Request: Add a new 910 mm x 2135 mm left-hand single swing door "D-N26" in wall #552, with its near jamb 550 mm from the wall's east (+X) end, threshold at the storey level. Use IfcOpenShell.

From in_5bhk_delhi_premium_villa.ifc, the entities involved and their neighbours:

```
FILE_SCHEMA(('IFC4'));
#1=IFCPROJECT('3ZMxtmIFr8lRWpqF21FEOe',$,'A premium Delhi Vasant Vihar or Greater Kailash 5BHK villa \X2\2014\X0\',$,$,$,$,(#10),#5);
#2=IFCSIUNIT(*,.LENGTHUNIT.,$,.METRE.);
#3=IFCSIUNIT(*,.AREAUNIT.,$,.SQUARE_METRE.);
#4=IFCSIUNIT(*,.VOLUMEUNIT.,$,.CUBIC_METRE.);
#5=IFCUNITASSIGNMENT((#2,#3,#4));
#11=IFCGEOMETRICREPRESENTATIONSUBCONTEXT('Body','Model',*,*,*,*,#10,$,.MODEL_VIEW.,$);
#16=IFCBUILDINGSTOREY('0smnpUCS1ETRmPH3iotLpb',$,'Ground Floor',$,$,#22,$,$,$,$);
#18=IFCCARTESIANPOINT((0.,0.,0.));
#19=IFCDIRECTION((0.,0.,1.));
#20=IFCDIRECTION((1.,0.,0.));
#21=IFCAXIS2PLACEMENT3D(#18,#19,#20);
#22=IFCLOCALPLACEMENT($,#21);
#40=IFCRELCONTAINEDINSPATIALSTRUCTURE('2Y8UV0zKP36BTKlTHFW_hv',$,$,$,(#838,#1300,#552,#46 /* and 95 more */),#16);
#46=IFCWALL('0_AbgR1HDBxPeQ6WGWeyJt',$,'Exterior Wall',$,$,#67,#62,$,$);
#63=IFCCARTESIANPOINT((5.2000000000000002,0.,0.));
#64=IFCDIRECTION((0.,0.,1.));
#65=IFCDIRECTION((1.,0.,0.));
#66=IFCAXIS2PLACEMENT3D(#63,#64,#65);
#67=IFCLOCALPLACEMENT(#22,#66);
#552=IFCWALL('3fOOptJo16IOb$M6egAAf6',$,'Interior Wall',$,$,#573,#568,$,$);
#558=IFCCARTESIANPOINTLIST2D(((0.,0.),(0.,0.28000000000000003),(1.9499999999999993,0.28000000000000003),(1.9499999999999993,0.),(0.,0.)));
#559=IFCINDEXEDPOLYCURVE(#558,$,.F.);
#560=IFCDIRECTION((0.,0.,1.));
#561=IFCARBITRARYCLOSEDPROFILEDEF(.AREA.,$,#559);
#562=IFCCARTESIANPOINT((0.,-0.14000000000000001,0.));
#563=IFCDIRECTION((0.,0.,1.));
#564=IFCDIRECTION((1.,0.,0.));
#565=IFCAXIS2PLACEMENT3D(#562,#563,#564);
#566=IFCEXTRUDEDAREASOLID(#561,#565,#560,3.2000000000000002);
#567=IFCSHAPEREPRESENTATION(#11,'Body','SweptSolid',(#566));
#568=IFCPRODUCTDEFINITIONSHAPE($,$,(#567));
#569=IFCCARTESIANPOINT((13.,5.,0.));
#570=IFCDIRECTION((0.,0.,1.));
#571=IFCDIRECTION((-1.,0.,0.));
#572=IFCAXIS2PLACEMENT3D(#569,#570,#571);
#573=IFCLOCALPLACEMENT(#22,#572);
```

```python
import numpy as np
import ifcopenshell
import ifcopenshell.api.feature
import ifcopenshell.api.geometry
import ifcopenshell.api.root
import ifcopenshell.api.spatial
import ifcopenshell.geom
import ifcopenshell.util.element
import ifcopenshell.util.placement
import ifcopenshell.util.representation
import ifcopenshell.util.shape
import ifcopenshell.util.unit

model = ifcopenshell.open("in_5bhk_delhi_premium_villa.ifc")
unit_scale = ifcopenshell.util.unit.calculate_unit_scale(model)
settings = ifcopenshell.geom.settings()


def volume(element):
    """Net volume in cubic metres, openings subtracted."""
    shape = ifcopenshell.geom.create_shape(settings, element)
    return ifcopenshell.util.shape.get_volume(shape.geometry)


wall = model.by_id(552)
storey = ifcopenshell.util.element.get_container(wall, ifc_class="IfcBuildingStorey")
context = ifcopenshell.util.representation.get_context(model, "Model", "Body", "MODEL_VIEW")
before = volume(wall)

width, height, from_end, sill = 0.91, 2.135, 0.55, 0.0  # metres

# The wall runs along its own X axis, and the end named is its -X end.
wall_shape = ifcopenshell.geom.create_shape(settings, wall)
x, y, z = ifcopenshell.util.shape.get_vertices(wall_shape.geometry).T
start = x.min() + from_end
face, thickness = float(y.min()), float(y.max() - y.min())
wall_matrix = ifcopenshell.util.placement.get_local_placement(wall.ObjectPlacement)
level = ifcopenshell.util.placement.get_local_placement(storey.ObjectPlacement)[2, 3]


def in_wall(x, y):
    """Placement at x, y metres in the wall's axes, at sill height."""
    matrix = wall_matrix.copy()
    matrix[:, 3] = wall_matrix @ np.array([x / unit_scale, y / unit_scale, 0.0, 1.0])
    matrix[2, 3] = level + sill / unit_scale
    return matrix


# Opening: a box that overshoots both wall faces by 50 mm.
opening = ifcopenshell.api.root.create_entity(model, ifc_class="IfcOpeningElement", predefined_type="OPENING")
box = ifcopenshell.api.geometry.add_wall_representation(
    model, context=context, length=width, height=height, thickness=thickness + 0.1
)
ifcopenshell.api.geometry.assign_representation(model, product=opening, representation=box)
ifcopenshell.api.geometry.edit_object_placement(model, product=opening, matrix=in_wall(start, face - 0.05), is_si=False)
ifcopenshell.api.feature.add_feature(model, feature=opening, element=wall)

door = ifcopenshell.api.root.create_entity(model, ifc_class="IfcDoor", name="D-N26", predefined_type="DOOR")
door.OverallWidth, door.OverallHeight = width / unit_scale, height / unit_scale
door.OperationType = "SINGLE_SWING_LEFT"
body = ifcopenshell.api.geometry.add_door_representation(
    model,
    context=context,
    overall_width=door.OverallWidth,
    overall_height=door.OverallHeight,
    operation_type="SINGLE_SWING_LEFT",
    lining_properties={"LiningDepth": thickness / unit_scale, "ThresholdDepth": thickness / unit_scale},
)
ifcopenshell.api.geometry.assign_representation(model, product=door, representation=body)
ifcopenshell.api.spatial.assign_container(model, products=[door], relating_structure=storey)
ifcopenshell.api.feature.add_filling(model, opening=opening, element=door)

# The lining spans the wall, so the door starts at the wall face.
ifcopenshell.api.geometry.edit_object_placement(model, product=door, matrix=in_wall(start, face), is_si=False)

after = volume(wall)

print(f"wall volume {before:.3f} -> {after:.3f} m3")

model.write("in_5bhk_delhi_premium_villa_updated.ifc")
```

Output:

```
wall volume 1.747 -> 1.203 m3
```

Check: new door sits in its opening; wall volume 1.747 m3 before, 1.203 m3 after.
